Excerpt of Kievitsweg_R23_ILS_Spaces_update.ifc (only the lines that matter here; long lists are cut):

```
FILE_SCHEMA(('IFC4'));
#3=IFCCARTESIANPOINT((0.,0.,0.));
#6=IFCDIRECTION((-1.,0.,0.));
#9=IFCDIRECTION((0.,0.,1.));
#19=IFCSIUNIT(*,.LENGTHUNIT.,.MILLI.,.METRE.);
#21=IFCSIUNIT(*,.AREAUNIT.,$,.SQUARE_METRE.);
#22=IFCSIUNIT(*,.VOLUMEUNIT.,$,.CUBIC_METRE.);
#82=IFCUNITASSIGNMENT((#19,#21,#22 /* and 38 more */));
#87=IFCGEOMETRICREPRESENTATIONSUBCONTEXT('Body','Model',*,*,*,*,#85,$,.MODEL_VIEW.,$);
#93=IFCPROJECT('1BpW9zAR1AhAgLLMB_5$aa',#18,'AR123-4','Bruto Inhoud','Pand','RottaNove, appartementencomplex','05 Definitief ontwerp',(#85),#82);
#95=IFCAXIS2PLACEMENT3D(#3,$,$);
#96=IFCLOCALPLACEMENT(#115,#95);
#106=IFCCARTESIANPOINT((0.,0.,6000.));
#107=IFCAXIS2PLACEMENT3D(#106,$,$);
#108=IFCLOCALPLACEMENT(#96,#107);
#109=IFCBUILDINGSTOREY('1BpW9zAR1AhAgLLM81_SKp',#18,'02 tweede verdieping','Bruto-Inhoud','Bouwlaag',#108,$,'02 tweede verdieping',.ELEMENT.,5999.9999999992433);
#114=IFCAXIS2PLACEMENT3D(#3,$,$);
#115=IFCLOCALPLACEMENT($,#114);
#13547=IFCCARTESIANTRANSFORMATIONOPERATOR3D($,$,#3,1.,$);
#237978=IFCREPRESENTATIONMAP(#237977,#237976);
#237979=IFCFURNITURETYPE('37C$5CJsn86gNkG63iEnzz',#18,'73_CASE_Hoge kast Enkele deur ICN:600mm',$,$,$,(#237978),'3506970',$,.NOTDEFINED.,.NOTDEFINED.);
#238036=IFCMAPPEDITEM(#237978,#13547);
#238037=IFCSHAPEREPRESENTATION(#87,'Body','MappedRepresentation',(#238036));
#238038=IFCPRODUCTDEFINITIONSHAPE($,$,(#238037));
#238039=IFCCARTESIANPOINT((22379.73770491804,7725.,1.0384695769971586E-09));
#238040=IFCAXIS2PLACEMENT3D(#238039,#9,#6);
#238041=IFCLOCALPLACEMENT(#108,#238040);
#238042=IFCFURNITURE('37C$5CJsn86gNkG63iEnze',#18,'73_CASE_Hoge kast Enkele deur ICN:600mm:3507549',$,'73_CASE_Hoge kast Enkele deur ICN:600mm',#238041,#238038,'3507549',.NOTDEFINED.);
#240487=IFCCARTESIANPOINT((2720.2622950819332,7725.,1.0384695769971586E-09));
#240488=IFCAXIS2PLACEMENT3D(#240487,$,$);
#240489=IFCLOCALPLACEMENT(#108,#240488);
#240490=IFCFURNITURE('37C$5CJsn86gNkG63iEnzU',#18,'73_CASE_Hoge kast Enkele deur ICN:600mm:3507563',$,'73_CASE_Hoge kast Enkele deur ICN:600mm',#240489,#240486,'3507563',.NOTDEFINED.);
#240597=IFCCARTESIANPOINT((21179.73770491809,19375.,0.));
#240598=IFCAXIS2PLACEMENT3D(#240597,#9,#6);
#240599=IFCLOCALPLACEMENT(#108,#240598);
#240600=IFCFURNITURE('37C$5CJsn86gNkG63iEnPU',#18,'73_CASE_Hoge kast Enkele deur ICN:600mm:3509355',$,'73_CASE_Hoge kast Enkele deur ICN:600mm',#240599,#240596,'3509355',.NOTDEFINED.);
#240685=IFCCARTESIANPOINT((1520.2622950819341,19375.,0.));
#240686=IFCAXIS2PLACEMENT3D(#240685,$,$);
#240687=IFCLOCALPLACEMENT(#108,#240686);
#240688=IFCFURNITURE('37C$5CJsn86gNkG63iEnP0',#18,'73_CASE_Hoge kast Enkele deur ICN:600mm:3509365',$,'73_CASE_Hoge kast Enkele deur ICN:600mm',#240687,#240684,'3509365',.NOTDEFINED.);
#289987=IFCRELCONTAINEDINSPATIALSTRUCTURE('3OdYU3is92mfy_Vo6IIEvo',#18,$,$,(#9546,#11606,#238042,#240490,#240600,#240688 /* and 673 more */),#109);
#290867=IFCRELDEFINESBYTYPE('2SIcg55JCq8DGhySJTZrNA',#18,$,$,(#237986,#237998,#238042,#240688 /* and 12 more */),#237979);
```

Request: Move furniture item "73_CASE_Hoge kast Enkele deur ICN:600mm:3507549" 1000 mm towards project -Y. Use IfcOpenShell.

```python
import ifcopenshell
import ifcopenshell.api.geometry
import ifcopenshell.util.placement

model = ifcopenshell.open("Kievitsweg_R23_ILS_Spaces_update.ifc")

item = model.by_id(238042)
matrix = ifcopenshell.util.placement.get_local_placement(item.ObjectPlacement)
matrix[1, 3] -= 1000.0
ifcopenshell.api.geometry.edit_object_placement(model, product=item, matrix=matrix, is_si=False)

print(ifcopenshell.util.placement.get_local_placement(item.ObjectPlacement).round(3) + 0.0)

model.write("Kievitsweg_R23_ILS_Spaces_update_rev.ifc")
```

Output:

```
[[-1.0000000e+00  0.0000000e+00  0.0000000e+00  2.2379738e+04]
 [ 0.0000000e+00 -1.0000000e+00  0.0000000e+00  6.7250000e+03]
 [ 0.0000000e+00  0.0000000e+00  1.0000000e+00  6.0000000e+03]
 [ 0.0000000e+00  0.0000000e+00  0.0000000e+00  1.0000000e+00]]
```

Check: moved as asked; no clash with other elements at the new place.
